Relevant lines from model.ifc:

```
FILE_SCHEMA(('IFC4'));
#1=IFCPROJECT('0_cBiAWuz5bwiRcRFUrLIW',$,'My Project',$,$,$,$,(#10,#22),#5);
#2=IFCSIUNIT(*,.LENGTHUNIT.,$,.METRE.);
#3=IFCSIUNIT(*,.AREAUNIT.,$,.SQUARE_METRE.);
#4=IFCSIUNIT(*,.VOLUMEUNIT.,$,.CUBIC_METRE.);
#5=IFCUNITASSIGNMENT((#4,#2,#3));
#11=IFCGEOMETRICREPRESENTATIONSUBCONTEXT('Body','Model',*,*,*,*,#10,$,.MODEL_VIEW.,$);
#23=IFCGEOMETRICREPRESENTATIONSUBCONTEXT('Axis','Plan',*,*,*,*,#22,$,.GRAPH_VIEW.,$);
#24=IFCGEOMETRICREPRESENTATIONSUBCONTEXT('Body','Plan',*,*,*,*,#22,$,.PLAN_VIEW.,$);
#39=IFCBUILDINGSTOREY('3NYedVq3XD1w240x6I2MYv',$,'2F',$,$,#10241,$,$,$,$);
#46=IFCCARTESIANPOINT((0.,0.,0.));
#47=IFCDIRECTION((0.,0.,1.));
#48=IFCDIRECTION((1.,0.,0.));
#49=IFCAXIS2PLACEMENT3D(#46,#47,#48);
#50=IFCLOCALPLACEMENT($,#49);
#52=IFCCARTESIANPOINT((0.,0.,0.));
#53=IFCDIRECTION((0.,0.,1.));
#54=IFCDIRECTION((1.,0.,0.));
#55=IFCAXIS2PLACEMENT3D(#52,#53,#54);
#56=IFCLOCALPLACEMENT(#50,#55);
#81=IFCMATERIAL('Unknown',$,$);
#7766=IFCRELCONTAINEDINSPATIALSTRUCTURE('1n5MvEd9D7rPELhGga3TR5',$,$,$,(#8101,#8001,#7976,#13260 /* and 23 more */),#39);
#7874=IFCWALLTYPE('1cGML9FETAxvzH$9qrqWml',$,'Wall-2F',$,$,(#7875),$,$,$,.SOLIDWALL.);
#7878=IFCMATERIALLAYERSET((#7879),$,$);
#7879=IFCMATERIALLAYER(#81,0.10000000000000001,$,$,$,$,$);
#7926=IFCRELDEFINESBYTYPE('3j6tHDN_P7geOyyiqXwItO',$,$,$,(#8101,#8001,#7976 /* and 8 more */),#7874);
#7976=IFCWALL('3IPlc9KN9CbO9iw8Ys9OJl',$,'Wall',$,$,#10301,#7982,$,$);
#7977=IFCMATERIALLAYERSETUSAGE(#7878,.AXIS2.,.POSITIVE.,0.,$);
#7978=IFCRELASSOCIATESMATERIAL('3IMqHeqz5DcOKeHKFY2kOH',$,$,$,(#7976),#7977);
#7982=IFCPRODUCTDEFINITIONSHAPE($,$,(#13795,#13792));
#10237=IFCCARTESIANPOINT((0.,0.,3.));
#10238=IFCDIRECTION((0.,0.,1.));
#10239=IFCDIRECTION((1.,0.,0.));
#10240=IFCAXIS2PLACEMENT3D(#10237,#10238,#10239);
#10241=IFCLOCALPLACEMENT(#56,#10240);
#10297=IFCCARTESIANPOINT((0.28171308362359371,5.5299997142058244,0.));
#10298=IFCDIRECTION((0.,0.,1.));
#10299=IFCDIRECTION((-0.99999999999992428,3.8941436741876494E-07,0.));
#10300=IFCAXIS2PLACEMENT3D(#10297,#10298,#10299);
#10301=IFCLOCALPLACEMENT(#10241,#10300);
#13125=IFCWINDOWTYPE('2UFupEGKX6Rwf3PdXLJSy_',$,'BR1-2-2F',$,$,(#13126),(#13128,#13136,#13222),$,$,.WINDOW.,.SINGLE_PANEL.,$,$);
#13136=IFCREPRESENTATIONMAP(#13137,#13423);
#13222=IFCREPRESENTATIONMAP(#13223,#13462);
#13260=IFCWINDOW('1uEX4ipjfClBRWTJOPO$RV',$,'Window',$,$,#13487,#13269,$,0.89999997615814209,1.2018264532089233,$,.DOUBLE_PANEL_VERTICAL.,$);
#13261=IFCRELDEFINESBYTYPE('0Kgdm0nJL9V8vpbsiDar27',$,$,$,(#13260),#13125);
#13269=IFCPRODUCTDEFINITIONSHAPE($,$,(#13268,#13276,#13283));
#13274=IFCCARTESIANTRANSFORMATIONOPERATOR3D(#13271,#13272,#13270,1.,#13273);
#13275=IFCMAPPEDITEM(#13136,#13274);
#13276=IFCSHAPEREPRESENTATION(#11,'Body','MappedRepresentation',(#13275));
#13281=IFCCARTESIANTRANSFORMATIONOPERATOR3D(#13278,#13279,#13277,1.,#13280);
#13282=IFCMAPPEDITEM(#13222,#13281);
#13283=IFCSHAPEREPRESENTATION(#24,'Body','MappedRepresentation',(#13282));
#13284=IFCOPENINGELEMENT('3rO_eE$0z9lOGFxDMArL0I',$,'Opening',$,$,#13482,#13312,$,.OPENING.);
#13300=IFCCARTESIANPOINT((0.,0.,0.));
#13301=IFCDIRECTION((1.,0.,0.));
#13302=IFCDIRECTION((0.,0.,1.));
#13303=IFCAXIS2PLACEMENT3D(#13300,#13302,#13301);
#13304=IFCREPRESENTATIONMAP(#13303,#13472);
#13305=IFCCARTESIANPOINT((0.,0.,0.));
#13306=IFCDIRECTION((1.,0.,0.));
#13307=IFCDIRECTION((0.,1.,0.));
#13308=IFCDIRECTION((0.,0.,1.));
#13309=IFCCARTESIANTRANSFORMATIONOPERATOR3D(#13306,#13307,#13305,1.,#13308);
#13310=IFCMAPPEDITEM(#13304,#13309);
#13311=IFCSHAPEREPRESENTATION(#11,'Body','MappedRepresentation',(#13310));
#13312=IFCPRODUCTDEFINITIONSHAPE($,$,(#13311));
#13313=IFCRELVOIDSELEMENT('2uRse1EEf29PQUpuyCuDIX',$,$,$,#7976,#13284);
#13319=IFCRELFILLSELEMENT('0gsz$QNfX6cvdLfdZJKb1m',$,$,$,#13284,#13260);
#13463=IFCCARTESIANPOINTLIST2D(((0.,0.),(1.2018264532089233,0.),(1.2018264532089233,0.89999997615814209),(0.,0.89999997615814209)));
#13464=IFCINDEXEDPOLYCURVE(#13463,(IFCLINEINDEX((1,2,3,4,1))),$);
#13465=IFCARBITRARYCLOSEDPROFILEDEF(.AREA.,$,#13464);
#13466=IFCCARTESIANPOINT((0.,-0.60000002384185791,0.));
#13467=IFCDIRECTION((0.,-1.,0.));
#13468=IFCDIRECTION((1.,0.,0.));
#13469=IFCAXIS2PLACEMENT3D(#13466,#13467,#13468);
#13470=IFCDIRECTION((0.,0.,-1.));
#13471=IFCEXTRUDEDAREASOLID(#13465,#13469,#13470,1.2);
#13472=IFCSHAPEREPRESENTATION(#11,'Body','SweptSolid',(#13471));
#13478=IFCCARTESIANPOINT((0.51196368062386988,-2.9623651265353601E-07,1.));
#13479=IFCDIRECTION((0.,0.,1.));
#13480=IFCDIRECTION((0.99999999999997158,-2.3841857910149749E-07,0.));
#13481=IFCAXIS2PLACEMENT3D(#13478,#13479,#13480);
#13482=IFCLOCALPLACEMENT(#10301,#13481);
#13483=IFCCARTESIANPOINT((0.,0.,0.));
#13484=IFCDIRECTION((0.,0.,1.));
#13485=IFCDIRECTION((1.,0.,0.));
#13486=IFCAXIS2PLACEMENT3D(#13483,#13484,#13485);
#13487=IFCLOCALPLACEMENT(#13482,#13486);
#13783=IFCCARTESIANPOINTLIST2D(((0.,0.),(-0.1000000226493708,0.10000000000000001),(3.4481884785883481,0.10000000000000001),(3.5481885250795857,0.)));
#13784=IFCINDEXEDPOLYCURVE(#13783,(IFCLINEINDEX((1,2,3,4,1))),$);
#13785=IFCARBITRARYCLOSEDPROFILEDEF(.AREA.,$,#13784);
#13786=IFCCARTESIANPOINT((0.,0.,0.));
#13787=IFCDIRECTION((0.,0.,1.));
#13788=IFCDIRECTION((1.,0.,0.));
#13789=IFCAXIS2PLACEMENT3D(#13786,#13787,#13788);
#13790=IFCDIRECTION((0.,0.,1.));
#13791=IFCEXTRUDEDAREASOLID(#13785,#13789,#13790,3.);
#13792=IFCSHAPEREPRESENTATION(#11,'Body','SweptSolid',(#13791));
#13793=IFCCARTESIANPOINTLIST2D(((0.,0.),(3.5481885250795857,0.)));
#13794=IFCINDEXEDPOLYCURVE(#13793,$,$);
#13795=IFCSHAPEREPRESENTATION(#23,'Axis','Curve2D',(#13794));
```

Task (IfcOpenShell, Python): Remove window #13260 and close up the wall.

```python
import ifcopenshell
import ifcopenshell.api.feature
import ifcopenshell.api.root
import ifcopenshell.geom
import ifcopenshell.util.shape

model = ifcopenshell.open("model.ifc")
settings = ifcopenshell.geom.settings()


def volume(element):
    """Net volume in cubic metres, openings subtracted."""
    shape = ifcopenshell.geom.create_shape(settings, element)
    return ifcopenshell.util.shape.get_volume(shape.geometry)


window = model.by_guid("1uEX4ipjfClBRWTJOPO$RV")
opening = window.FillsVoids[0].RelatingOpeningElement
wall = opening.VoidsElements[0].RelatingBuildingElement
before = volume(wall)

ifcopenshell.api.root.remove_product(model, product=window)
ifcopenshell.api.feature.remove_feature(model, feature=opening)

after = volume(wall)

print(f"wall volume {before:.3f} -> {after:.3f} m3")

model.write("model_rev.ifc")
```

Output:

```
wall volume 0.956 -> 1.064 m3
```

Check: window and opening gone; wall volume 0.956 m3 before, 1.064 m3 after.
